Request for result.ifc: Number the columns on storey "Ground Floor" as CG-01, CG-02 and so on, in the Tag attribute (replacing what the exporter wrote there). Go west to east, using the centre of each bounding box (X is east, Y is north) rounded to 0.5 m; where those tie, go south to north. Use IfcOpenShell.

First a look at what the model holds.

```python
import ifcopenshell
import ifcopenshell.util.element
import ifcopenshell.util.placement

model = ifcopenshell.open("result.ifc")
print(model.schema)
storey = next(s for s in model.by_type("IfcBuildingStorey") if s.Name == "Ground Floor")
columns = [e for e in ifcopenshell.util.element.get_decomposition(storey) if e.is_a("IfcColumn")]
for e in sorted(columns, key=lambda e: e.id()):
    origin = ifcopenshell.util.placement.get_local_placement(e.ObjectPlacement)[:3, 3]
    print(e.id(), e.Tag, e.Name, origin.round(2) + 0.0, sep=" | ")
```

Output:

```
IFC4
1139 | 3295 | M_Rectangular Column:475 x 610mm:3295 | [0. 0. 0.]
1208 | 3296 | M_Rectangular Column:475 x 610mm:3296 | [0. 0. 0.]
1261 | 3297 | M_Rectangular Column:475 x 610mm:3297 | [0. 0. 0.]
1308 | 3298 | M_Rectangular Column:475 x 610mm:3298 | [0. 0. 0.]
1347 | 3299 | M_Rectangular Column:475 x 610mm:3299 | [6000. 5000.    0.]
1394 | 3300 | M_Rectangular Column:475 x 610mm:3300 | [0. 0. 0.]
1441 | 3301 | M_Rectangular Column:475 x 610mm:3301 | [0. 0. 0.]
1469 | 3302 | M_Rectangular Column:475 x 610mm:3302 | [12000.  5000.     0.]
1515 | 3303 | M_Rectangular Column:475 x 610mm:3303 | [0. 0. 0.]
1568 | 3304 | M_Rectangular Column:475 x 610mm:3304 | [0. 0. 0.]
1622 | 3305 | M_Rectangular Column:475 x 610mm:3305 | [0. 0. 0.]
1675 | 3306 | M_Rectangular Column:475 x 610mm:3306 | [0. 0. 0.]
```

```python
import ifcopenshell
import ifcopenshell.geom
import ifcopenshell.util.element
import ifcopenshell.util.shape

model = ifcopenshell.open("result.ifc")
settings = ifcopenshell.geom.settings()
settings.set("use-world-coords", True)


def centre(element):
    shape = ifcopenshell.geom.create_shape(settings, element)
    return ifcopenshell.util.shape.get_bbox_centroid(shape.geometry)


storey = next(s for s in model.by_type("IfcBuildingStorey") if s.Name == "Ground Floor")
columns = [e for e in ifcopenshell.util.element.get_decomposition(storey) if e.is_a("IfcColumn")]

# Insertion points can sit at a corner or the storey origin, so sort by the geometry (in metres).
centres = {e: centre(e) for e in columns}
columns.sort(key=lambda e: (round(centres[e][0] / 0.5), centres[e][1]))

for i, e in enumerate(columns, start=1):
    number = f"CG-{i:02d}"
    e.Tag = number
    print(e.id(), number)

model.write("result_v2.ifc")
```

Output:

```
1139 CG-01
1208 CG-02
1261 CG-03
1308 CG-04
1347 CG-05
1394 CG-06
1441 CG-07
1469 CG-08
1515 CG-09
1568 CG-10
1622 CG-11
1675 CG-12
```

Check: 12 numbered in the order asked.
